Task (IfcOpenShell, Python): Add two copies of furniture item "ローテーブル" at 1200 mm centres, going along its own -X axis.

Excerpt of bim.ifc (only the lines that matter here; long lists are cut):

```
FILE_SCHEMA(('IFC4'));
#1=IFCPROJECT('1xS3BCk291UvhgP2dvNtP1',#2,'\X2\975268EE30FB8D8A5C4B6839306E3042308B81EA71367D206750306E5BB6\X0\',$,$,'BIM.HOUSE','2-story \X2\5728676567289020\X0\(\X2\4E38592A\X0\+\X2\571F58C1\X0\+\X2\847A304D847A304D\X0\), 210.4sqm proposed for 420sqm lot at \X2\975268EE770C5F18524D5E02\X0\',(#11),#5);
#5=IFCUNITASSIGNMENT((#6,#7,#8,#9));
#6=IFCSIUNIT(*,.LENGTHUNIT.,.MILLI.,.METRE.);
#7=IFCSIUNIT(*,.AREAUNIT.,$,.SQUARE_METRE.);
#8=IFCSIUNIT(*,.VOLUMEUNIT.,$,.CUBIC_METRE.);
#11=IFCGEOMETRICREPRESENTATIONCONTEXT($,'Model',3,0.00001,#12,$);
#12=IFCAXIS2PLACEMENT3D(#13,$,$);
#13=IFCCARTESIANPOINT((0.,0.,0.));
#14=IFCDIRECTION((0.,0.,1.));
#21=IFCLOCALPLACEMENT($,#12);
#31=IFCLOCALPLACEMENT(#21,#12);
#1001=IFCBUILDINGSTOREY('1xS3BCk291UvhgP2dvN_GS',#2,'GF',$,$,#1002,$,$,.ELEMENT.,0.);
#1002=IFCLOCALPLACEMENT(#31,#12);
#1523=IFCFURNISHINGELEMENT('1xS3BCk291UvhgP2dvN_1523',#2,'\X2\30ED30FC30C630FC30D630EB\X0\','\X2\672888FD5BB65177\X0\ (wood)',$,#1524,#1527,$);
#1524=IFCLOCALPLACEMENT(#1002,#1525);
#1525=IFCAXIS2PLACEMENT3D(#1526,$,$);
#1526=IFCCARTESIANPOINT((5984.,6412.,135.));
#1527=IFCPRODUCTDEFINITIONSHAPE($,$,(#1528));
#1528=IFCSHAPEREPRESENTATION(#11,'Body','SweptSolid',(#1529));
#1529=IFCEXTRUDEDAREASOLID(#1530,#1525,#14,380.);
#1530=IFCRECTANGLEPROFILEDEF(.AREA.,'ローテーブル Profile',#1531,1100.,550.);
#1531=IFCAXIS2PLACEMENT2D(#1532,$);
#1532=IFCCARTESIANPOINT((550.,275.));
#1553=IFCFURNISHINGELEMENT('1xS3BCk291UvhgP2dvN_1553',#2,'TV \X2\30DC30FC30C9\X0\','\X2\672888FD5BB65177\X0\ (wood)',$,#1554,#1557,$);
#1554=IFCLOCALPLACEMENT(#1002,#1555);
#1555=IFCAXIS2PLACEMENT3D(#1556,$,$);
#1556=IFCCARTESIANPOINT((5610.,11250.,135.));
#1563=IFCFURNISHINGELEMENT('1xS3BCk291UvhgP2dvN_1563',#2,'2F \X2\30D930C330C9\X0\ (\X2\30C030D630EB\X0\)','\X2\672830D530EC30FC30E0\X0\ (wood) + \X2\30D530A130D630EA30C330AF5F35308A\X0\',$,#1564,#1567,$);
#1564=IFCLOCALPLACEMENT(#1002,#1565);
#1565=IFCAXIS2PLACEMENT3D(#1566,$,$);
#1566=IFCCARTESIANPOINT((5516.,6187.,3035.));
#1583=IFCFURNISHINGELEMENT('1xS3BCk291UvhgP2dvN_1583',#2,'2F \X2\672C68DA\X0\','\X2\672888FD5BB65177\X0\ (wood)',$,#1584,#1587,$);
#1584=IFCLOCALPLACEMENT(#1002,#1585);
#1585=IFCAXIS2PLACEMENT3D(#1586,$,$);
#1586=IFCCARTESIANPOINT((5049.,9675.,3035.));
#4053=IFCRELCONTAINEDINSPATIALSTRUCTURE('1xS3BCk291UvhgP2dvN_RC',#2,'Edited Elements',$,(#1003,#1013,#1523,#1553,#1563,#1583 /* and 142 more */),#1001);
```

```python
import ifcopenshell
import ifcopenshell.api.geometry
import ifcopenshell.api.root
import ifcopenshell.util.element
import ifcopenshell.util.placement

model = ifcopenshell.open("bim.ifc")


def reuse_history(source, copy):
    """copy_class also copies each property set's owner history, people and application; keep the originals."""
    for rel in copy.IsDefinedBy:
        if rel.is_a("IfcRelDefinesByProperties") and (history := rel.RelatingPropertyDefinition.OwnerHistory):
            rel.RelatingPropertyDefinition.OwnerHistory = source.OwnerHistory
            ifcopenshell.util.element.remove_deep2(model, history)


source = model.by_guid("1xS3BCk291UvhgP2dvN_1523")
base = ifcopenshell.util.placement.get_local_placement(source.ObjectPlacement)
step = -base[:3, 0] * 1200.0

for i in range(1, 3):
    copy = ifcopenshell.api.root.copy_class(model, product=source)
    copy.Representation = ifcopenshell.util.element.copy_deep(
        model, source.Representation, exclude=["IfcGeometricRepresentationContext", "IfcRepresentationMap"]
    )
    reuse_history(source, copy)
    matrix = base.copy()
    matrix[:3, 3] += i * step
    print("added at", matrix[:3, 3].round(3) + 0.0)
    ifcopenshell.api.geometry.edit_object_placement(model, product=copy, matrix=matrix, is_si=False)

model.write("bim_rev.ifc")
```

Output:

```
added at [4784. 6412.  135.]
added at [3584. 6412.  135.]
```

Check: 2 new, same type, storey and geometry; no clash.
